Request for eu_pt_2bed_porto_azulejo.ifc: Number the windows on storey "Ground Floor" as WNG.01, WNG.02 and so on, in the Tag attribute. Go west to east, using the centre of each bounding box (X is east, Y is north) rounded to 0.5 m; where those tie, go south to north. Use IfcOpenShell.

First a look at what the model holds.

```python
import ifcopenshell
import ifcopenshell.util.element
import ifcopenshell.util.placement

model = ifcopenshell.open("eu_pt_2bed_porto_azulejo.ifc")
print(model.schema)
storey = next(s for s in model.by_type("IfcBuildingStorey") if s.Name == "Ground Floor")
windows = [e for e in ifcopenshell.util.element.get_decomposition(storey) if e.is_a("IfcWindow")]
for e in sorted(windows, key=lambda e: e.id()):
    origin = ifcopenshell.util.placement.get_local_placement(e.ObjectPlacement)[:3, 3]
    print(e.id(), e.Tag, e.Name, origin.round(2) + 0.0, sep=" | ")
```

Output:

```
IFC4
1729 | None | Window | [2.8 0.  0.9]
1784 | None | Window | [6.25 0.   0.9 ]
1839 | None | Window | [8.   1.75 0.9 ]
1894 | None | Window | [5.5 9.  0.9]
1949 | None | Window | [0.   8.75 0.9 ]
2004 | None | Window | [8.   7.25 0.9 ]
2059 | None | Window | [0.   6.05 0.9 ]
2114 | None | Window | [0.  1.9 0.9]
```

```python
import ifcopenshell
import ifcopenshell.geom
import ifcopenshell.util.element
import ifcopenshell.util.shape

model = ifcopenshell.open("eu_pt_2bed_porto_azulejo.ifc")
settings = ifcopenshell.geom.settings()
settings.set("use-world-coords", True)


def centre(element):
    shape = ifcopenshell.geom.create_shape(settings, element)
    return ifcopenshell.util.shape.get_bbox_centroid(shape.geometry)


storey = next(s for s in model.by_type("IfcBuildingStorey") if s.Name == "Ground Floor")
windows = [e for e in ifcopenshell.util.element.get_decomposition(storey) if e.is_a("IfcWindow")]

# Insertion points can sit at a corner or the storey origin, so sort by the geometry (in metres).
centres = {e: centre(e) for e in windows}
windows.sort(key=lambda e: (round(centres[e][0] / 0.5), centres[e][1]))

for i, e in enumerate(windows, start=1):
    number = f"WNG.{i:02d}"
    e.Tag = number
    print(e.id(), number)

model.write("eu_pt_2bed_porto_azulejo-out.ifc")
```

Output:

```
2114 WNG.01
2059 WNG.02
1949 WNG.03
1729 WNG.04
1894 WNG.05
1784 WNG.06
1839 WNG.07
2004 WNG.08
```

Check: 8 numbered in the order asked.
